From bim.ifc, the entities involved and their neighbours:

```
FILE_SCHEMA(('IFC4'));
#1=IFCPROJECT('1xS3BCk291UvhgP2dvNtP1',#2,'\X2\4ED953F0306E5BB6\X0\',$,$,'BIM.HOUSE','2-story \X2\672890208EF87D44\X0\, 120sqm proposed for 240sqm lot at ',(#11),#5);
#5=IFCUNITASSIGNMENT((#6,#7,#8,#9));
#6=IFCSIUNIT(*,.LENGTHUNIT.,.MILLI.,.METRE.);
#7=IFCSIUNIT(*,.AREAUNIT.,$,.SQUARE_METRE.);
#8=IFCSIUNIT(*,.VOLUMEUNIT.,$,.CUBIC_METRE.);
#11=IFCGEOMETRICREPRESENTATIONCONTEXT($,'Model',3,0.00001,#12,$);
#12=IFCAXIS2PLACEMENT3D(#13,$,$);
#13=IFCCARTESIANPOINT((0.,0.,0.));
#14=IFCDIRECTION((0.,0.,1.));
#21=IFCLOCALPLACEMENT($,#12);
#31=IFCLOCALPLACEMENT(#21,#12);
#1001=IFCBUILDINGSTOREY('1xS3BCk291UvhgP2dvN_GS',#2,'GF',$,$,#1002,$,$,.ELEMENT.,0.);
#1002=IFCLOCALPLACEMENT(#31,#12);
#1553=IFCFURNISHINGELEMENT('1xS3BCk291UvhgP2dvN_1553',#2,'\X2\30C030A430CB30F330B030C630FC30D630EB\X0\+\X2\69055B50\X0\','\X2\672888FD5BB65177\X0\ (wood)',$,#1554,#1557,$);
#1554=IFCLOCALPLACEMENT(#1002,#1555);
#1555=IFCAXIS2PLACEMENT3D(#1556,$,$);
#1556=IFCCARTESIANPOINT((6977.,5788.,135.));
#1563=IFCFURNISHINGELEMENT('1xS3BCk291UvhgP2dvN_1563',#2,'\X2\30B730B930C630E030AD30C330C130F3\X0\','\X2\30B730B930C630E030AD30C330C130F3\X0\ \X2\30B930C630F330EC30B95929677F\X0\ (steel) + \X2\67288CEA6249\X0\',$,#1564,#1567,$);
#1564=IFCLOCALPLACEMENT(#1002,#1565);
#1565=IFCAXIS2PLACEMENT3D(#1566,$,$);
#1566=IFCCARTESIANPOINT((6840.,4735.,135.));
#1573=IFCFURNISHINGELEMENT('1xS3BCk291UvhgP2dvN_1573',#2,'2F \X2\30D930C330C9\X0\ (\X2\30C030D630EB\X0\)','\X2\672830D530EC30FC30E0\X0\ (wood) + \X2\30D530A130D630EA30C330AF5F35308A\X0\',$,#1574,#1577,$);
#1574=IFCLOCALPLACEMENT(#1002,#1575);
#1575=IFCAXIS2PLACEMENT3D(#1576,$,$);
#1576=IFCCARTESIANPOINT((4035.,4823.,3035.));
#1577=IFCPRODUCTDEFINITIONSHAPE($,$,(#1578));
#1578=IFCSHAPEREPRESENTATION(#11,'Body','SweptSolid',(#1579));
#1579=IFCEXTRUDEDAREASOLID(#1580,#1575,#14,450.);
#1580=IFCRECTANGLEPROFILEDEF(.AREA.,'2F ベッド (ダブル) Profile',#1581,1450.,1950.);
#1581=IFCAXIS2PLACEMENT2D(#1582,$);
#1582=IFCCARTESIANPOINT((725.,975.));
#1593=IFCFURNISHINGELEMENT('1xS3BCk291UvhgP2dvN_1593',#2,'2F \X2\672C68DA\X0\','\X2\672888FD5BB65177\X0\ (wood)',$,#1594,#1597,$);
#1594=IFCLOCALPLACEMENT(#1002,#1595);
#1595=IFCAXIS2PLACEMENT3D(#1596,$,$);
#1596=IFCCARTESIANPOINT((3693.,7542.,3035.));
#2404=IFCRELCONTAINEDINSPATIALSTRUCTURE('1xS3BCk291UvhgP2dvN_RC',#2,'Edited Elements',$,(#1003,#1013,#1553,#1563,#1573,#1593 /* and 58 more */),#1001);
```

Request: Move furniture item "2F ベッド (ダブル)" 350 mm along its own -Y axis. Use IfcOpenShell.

```python
import ifcopenshell
import ifcopenshell.api.geometry
import ifcopenshell.util.placement
import ifcopenshell.util.unit

model = ifcopenshell.open("bim.ifc")
unit_scale = ifcopenshell.util.unit.calculate_unit_scale(model)

item = model.by_guid("1xS3BCk291UvhgP2dvN_1573")
matrix = ifcopenshell.util.placement.get_local_placement(item.ObjectPlacement)
matrix[:3, 3] -= matrix[:3, 1] * 0.35 / unit_scale
ifcopenshell.api.geometry.edit_object_placement(model, product=item, matrix=matrix, is_si=False)

print(ifcopenshell.util.placement.get_local_placement(item.ObjectPlacement).round(3) + 0.0)

model.write("bim-out.ifc")
```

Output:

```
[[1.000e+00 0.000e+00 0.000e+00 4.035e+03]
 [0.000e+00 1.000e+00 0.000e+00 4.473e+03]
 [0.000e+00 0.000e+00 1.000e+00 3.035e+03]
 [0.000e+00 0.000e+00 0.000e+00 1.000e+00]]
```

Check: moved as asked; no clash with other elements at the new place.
